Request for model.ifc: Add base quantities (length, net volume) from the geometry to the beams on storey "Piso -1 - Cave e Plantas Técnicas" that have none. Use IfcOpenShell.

First a look at what the model holds.

```python
import ifcopenshell
import ifcopenshell.util.element
import ifcopenshell.util.unit

model = ifcopenshell.open("model.ifc")
print(model.schema)
for unit_type in ("LENGTHUNIT", "AREAUNIT", "VOLUMEUNIT"):
    print(unit_type, ifcopenshell.util.unit.calculate_unit_scale(model, unit_type))
storey = next(s for s in model.by_type("IfcBuildingStorey") if s.Name == "Piso -1 - Cave e Plantas Técnicas")
beams = [e for e in ifcopenshell.util.element.get_decomposition(storey) if e.is_a("IfcBeam")]
for e in sorted(beams, key=lambda e: e.id()):
    print(e.id(), e.is_a(), e.Name, list(ifcopenshell.util.element.get_psets(e, qtos_only=True)), sep=" | ")
```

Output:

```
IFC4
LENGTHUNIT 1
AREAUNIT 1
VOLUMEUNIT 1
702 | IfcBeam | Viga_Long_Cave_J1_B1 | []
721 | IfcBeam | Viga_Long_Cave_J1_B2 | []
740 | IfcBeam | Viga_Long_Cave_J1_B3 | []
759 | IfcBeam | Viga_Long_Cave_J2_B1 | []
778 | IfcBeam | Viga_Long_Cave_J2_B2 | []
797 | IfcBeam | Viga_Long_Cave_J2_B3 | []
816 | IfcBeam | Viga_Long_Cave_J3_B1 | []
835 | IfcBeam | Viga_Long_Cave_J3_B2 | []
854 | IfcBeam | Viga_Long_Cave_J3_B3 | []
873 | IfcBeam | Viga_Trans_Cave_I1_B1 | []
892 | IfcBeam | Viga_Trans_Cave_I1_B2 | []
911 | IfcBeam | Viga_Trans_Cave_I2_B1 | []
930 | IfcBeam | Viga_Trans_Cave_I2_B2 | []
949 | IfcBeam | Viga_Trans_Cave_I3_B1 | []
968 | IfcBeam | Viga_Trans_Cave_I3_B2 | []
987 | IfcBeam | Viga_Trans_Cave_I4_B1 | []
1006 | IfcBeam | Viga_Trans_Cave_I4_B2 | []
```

```python
import ifcopenshell
import ifcopenshell.api.pset
import ifcopenshell.geom
import ifcopenshell.util.element
import ifcopenshell.util.shape
import ifcopenshell.util.unit

model = ifcopenshell.open("model.ifc")
unit_scale = ifcopenshell.util.unit.calculate_unit_scale(model)
volume_scale = ifcopenshell.util.unit.calculate_unit_scale(model, "VOLUMEUNIT")
settings = ifcopenshell.geom.settings()

storey = next(s for s in model.by_type("IfcBuildingStorey") if s.Name == "Piso -1 - Cave e Plantas Técnicas")
beams = [e for e in ifcopenshell.util.element.get_decomposition(storey) if e.is_a("IfcBeam")]

for e in sorted(beams, key=lambda e: e.id()):
    if ifcopenshell.util.element.get_psets(e, qtos_only=True, should_inherit=False):
        continue
    # Geometry comes back in metres, in the element's own axes.
    shape = ifcopenshell.geom.create_shape(settings, e)
    values = {
        "Length": ifcopenshell.util.shape.get_max_xyz(shape.geometry) / unit_scale,
        "NetVolume": ifcopenshell.util.shape.get_volume(shape.geometry) / volume_scale,
    }
    qto = ifcopenshell.api.pset.add_qto(model, product=e, name="Qto_BeamBaseQuantities")
    ifcopenshell.api.pset.edit_qto(model, qto=qto, properties=values)
    print(e.id(), {k: round(v, 3) for k, v in values.items()})

model.write("model_rev.ifc")
```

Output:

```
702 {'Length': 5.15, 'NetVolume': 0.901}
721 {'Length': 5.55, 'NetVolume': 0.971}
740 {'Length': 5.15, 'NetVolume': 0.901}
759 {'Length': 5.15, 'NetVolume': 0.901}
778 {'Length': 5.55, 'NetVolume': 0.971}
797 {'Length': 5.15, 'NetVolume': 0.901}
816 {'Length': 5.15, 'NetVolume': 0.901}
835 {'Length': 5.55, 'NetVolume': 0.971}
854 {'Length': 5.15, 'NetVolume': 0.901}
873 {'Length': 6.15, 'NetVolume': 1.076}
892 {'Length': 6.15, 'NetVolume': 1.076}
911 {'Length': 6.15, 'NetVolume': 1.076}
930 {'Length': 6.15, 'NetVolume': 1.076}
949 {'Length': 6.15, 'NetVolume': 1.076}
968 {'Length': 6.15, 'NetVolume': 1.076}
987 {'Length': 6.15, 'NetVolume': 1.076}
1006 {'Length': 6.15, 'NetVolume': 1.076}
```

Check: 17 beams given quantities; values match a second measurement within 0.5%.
